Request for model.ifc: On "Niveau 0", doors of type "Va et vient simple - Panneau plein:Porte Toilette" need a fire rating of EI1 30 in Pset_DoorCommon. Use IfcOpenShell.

First a look at what the model holds.

```python
import ifcopenshell
import ifcopenshell.util.element

model = ifcopenshell.open("model.ifc")
print(model.schema)
storey = next(s for s in model.by_type("IfcBuildingStorey") if s.Name == "Niveau 0")
doors = [e for e in ifcopenshell.util.element.get_decomposition(storey) if e.is_a("IfcDoor")]
seen = {}
for e in doors:
    element_type = ifcopenshell.util.element.get_type(e)
    key = (element_type.Name if element_type != e and element_type else None, ifcopenshell.util.element.get_pset(e, "Pset_DoorCommon", "FireRating"))
    seen[key] = seen.get(key, 0) + 1
for (name, value), count in sorted(seen.items(), key=str):
    print(count, "x", name, "|", value)
```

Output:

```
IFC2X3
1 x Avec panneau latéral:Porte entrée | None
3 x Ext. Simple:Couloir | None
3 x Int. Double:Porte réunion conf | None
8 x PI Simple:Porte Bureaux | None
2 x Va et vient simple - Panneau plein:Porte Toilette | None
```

```python
import ifcopenshell
import ifcopenshell.api.pset
import ifcopenshell.util.element

model = ifcopenshell.open("model.ifc")

storey = next(s for s in model.by_type("IfcBuildingStorey") if s.Name == "Niveau 0")
doors = [e for e in ifcopenshell.util.element.get_decomposition(storey) if e.is_a("IfcDoor")]

count = 0
for e in doors:
    element_type = ifcopenshell.util.element.get_type(e)
    if element_type in (None, e) or element_type.Name != "Va et vient simple - Panneau plein:Porte Toilette":
        continue
    # add_pset returns the element's existing set when there is one.
    pset = ifcopenshell.api.pset.add_pset(model, product=e, name="Pset_DoorCommon")
    ifcopenshell.api.pset.edit_pset(model, pset=pset, properties={"FireRating": "EI1 30"})
    count += 1

print(count, "doors updated")

model.write("model_updated.ifc")
```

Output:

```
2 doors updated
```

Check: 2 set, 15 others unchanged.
